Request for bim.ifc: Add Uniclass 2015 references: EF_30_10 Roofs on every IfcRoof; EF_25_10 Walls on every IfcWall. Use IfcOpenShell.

First a look at what the model holds.

```python
import ifcopenshell

model = ifcopenshell.open("bim.ifc")
print(model.schema)
print("classifications:", [c.Name for c in model.by_type("IfcClassification")])
for ifc_class in ("IfcDoor", "IfcRoof", "IfcStair", "IfcWall", "IfcWindow"):
    print(ifc_class, len(model.by_type(ifc_class)))
```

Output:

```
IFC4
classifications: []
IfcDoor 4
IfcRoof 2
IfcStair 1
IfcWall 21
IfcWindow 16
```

```python
import ifcopenshell
import ifcopenshell.api.classification

model = ifcopenshell.open("bim.ifc")

system = ifcopenshell.api.classification.add_classification(model, classification="Uniclass 2015")

codes = {
    "IfcRoof": ("EF_30_10", "Roofs"),
    "IfcWall": ("EF_25_10", "Walls"),
}
for ifc_class, (code, name) in codes.items():
    products = model.by_type(ifc_class)
    ifcopenshell.api.classification.add_reference(
        model, products=products, classification=system, identification=code, name=name
    )
    print(code, len(products))

model.write("bim_v2.ifc")
```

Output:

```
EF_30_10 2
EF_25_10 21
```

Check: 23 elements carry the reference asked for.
